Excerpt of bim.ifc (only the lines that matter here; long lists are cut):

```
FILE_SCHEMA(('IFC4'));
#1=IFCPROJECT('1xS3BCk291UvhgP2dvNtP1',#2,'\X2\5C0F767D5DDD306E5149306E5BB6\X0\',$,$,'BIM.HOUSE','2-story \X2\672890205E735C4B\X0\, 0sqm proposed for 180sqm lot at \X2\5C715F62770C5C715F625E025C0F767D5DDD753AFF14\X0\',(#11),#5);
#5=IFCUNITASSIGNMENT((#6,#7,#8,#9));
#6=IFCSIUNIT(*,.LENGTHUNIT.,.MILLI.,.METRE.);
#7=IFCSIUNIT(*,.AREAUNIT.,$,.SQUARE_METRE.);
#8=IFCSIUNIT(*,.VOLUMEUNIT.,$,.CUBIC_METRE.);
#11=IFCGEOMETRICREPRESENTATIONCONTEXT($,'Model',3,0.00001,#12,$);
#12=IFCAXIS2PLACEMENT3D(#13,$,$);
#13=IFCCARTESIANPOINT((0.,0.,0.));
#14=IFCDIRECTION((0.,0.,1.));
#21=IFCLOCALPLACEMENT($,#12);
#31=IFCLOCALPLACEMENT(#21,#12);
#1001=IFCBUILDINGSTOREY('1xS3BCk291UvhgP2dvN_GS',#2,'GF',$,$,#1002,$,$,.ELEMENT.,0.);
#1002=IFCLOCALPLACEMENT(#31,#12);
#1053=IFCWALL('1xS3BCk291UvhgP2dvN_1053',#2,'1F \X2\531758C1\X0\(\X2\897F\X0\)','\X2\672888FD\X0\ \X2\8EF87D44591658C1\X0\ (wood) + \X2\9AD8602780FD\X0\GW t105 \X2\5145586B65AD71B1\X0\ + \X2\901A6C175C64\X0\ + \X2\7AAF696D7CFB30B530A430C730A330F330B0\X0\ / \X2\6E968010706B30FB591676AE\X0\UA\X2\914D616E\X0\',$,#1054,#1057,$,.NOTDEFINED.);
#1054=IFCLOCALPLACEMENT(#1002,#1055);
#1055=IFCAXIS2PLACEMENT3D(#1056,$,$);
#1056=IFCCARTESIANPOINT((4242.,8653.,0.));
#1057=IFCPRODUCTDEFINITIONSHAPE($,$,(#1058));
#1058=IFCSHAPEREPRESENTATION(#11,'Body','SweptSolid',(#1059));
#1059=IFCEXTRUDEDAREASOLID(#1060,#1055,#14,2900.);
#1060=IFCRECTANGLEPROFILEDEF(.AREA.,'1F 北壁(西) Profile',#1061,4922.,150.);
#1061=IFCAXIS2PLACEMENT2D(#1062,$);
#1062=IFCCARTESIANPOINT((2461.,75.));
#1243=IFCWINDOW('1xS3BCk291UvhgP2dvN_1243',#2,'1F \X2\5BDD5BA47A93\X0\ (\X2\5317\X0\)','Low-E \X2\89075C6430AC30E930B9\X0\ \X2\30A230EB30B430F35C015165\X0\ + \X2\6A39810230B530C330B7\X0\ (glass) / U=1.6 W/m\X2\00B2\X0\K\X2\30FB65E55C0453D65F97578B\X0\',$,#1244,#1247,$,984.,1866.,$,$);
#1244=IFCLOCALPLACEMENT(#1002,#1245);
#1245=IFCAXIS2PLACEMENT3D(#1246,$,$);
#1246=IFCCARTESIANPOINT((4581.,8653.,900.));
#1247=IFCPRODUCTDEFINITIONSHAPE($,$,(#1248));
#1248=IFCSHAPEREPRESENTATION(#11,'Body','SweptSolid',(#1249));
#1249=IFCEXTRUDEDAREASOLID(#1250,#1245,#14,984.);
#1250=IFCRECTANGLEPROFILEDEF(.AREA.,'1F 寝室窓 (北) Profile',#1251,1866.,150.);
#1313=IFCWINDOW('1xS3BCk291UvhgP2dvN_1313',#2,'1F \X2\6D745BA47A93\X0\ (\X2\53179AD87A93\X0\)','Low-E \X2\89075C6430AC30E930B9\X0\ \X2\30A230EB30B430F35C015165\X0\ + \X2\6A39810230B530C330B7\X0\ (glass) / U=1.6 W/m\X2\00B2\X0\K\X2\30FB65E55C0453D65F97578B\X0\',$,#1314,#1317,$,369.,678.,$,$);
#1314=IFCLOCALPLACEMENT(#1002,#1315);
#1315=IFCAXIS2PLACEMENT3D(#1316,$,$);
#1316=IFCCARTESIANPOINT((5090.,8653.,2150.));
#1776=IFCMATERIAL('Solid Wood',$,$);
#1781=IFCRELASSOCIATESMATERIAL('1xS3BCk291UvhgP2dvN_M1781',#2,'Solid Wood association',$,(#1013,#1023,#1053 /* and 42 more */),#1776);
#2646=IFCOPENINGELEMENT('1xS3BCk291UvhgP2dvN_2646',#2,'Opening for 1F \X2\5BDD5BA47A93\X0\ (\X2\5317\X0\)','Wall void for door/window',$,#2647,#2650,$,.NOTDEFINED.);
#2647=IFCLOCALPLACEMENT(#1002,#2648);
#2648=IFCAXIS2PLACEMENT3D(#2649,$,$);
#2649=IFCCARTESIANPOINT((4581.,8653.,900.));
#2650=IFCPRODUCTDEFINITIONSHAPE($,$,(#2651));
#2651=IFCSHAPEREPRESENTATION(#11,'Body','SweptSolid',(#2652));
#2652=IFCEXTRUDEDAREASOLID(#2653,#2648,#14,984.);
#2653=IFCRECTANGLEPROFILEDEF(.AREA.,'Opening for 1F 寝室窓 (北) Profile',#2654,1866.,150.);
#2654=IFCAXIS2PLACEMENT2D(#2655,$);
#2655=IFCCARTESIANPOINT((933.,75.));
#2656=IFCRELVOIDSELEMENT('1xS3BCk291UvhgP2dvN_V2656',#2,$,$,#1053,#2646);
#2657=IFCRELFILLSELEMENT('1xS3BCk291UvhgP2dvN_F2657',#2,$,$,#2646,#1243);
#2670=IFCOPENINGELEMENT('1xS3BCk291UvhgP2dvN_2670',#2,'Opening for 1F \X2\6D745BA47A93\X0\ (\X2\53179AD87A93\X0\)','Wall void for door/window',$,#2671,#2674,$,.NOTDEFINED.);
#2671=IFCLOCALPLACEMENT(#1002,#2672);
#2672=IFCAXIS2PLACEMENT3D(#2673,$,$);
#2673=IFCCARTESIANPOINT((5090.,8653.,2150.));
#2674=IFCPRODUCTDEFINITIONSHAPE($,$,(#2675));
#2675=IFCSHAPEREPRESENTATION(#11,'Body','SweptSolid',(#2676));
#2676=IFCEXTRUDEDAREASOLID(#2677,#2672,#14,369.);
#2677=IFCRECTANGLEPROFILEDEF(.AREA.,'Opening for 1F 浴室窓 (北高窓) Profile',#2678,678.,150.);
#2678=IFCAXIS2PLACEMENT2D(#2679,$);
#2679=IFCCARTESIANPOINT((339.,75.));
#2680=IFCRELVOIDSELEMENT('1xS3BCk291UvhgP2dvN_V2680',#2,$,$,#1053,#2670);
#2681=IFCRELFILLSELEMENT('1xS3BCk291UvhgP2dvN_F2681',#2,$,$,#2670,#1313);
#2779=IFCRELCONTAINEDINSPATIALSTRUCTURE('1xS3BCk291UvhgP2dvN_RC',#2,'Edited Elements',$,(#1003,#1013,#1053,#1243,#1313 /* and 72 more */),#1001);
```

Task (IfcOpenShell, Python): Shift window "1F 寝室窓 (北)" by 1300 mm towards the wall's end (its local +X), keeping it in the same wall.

```python
import ifcopenshell
import ifcopenshell.api.geometry
import ifcopenshell.util.placement

model = ifcopenshell.open("bim.ifc")

window = model.by_guid("1xS3BCk291UvhgP2dvN_1243")
opening = window.FillsVoids[0].RelatingOpeningElement
wall = opening.VoidsElements[0].RelatingBuildingElement

wall_matrix = ifcopenshell.util.placement.get_local_placement(wall.ObjectPlacement)
shift = wall_matrix[:3, 0] * 1300.0
before = ifcopenshell.util.placement.get_local_placement(window.ObjectPlacement)[:3, 3].copy()

# The window is not placed relative to its opening, so move both.
for product in (opening, window):
    matrix = ifcopenshell.util.placement.get_local_placement(product.ObjectPlacement)
    matrix[:3, 3] += shift
    ifcopenshell.api.geometry.edit_object_placement(model, product=product, matrix=matrix, is_si=False)

after = ifcopenshell.util.placement.get_local_placement(window.ObjectPlacement)[:3, 3]
print("window moved by", (after - before).round(3) + 0.0)

model.write("bim_edited.ifc")
```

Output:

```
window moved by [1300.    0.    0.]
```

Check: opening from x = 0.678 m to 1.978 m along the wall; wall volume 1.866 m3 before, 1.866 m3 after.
